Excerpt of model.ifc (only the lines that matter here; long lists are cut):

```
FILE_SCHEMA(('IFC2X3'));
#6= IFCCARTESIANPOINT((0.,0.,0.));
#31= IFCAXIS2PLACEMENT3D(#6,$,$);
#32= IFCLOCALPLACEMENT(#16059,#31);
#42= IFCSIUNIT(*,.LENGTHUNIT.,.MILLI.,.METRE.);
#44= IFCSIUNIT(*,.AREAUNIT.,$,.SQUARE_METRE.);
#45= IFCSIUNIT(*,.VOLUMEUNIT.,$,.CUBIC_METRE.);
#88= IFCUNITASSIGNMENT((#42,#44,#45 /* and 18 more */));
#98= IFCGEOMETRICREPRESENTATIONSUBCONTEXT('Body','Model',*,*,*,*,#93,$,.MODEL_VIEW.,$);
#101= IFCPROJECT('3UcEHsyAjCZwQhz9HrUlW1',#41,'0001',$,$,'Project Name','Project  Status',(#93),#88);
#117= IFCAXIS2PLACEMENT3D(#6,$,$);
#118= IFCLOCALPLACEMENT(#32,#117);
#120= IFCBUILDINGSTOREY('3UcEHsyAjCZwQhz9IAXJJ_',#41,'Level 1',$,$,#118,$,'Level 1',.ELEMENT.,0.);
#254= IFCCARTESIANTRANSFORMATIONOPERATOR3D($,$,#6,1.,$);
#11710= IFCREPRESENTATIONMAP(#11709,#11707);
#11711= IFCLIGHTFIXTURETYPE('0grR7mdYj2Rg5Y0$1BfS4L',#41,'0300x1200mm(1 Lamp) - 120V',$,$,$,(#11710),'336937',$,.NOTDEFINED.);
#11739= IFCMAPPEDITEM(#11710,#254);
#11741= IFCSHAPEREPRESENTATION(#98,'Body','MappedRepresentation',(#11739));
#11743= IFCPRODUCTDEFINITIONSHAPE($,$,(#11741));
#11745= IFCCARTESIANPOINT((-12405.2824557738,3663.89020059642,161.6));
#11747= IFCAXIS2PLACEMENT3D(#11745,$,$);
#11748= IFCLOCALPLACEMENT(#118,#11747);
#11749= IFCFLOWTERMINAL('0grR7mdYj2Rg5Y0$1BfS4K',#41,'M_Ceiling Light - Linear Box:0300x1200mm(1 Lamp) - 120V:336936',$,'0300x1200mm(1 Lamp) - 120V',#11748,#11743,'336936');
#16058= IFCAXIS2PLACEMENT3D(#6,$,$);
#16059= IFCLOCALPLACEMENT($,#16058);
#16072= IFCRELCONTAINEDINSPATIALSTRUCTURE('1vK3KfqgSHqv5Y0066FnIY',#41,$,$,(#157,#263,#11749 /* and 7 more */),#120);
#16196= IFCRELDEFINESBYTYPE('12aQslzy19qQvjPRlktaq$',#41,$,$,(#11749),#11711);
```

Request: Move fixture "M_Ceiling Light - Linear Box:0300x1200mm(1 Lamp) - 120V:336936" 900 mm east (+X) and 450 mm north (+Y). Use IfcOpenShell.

```python
import ifcopenshell
import ifcopenshell.api.geometry
import ifcopenshell.util.placement
import ifcopenshell.util.unit

model = ifcopenshell.open("model.ifc")
unit_scale = ifcopenshell.util.unit.calculate_unit_scale(model)

item = model.by_guid("0grR7mdYj2Rg5Y0$1BfS4K")
matrix = ifcopenshell.util.placement.get_local_placement(item.ObjectPlacement)
matrix[0, 3] += 0.9 / unit_scale
matrix[1, 3] += 0.45 / unit_scale
ifcopenshell.api.geometry.edit_object_placement(model, product=item, matrix=matrix, is_si=False)

print(ifcopenshell.util.placement.get_local_placement(item.ObjectPlacement).round(3) + 0.0)

model.write("model_rev.ifc")
```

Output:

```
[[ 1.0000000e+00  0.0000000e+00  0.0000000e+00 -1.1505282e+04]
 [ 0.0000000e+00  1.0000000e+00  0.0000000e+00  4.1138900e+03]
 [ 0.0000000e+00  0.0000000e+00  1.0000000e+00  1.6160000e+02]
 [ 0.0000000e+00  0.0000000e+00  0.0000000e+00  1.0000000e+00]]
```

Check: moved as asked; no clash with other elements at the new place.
